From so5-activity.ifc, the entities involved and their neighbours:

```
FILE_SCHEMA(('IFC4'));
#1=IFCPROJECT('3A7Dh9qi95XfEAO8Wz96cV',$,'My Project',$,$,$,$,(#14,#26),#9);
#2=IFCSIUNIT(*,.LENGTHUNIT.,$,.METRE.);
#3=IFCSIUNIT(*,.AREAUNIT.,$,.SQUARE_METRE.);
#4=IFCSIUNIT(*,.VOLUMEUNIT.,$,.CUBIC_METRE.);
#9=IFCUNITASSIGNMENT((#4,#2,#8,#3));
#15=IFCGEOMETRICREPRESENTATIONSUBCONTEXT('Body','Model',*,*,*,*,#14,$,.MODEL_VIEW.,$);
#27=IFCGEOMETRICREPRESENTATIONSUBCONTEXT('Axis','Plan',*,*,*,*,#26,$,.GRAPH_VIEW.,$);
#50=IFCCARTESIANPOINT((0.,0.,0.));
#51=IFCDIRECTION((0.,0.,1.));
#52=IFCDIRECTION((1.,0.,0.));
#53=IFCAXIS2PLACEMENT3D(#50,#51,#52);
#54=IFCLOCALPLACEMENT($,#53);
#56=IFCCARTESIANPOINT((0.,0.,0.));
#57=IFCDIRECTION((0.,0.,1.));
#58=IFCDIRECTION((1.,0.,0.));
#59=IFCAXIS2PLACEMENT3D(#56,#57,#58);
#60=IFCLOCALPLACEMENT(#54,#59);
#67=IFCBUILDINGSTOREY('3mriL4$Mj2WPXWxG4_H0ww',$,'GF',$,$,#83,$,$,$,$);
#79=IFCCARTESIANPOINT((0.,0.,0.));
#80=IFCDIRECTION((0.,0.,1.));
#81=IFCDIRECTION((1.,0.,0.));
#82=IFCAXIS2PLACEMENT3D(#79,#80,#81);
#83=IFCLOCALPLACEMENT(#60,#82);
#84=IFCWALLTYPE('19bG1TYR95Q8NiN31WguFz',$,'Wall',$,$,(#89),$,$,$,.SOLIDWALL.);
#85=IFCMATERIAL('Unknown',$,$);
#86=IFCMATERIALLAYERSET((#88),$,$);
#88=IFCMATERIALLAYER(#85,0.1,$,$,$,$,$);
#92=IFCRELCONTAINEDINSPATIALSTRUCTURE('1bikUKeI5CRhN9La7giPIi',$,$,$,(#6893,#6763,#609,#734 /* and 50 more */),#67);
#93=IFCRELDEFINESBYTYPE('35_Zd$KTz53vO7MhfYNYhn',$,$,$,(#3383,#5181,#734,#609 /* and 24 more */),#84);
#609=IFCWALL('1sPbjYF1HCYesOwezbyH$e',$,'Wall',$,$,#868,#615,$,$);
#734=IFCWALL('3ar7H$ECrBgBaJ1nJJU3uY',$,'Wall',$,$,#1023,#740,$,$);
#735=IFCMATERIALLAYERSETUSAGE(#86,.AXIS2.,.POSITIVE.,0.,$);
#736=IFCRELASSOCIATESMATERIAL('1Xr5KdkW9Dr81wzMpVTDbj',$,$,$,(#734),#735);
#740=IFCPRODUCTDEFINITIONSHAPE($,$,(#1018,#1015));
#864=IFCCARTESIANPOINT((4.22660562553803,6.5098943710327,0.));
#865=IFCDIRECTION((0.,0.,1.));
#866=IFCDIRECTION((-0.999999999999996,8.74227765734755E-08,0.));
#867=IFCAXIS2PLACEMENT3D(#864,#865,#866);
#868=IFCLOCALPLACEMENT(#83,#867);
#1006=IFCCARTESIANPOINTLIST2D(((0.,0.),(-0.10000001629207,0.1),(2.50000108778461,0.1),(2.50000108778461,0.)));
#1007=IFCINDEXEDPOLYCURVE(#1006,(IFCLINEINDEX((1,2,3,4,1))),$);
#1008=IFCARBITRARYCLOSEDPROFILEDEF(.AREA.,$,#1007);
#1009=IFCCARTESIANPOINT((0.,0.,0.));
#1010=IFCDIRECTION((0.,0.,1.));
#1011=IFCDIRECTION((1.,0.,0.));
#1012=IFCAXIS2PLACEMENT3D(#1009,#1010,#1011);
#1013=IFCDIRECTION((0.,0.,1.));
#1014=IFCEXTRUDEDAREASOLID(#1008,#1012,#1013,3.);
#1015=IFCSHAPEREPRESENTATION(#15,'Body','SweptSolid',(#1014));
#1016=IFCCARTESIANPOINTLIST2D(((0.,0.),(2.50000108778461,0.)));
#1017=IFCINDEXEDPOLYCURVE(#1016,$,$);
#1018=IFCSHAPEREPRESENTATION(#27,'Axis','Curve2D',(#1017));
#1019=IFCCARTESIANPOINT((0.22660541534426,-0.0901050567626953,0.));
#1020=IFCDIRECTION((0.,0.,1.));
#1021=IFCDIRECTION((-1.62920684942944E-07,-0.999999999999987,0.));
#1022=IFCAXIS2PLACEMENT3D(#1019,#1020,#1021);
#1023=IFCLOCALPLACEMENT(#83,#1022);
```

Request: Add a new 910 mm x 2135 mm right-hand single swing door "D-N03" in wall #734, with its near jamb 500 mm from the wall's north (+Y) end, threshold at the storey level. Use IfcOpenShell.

```python
import numpy as np
import ifcopenshell
import ifcopenshell.api.feature
import ifcopenshell.api.geometry
import ifcopenshell.api.root
import ifcopenshell.api.spatial
import ifcopenshell.geom
import ifcopenshell.util.element
import ifcopenshell.util.placement
import ifcopenshell.util.representation
import ifcopenshell.util.shape
import ifcopenshell.util.unit

model = ifcopenshell.open("so5-activity.ifc")
unit_scale = ifcopenshell.util.unit.calculate_unit_scale(model)
settings = ifcopenshell.geom.settings()


def volume(element):
    """Net volume in cubic metres, openings subtracted."""
    shape = ifcopenshell.geom.create_shape(settings, element)
    return ifcopenshell.util.shape.get_volume(shape.geometry)


wall = model.by_id(734)
storey = ifcopenshell.util.element.get_container(wall, ifc_class="IfcBuildingStorey")
context = ifcopenshell.util.representation.get_context(model, "Model", "Body", "MODEL_VIEW")
before = volume(wall)

width, height, from_end, sill = 0.91, 2.135, 0.5, 0.0  # metres

# The wall runs along its own X axis, and the end named is its -X end.
wall_shape = ifcopenshell.geom.create_shape(settings, wall)
x, y, z = ifcopenshell.util.shape.get_vertices(wall_shape.geometry).T
start = x.min() + from_end
face, thickness = float(y.min()), float(y.max() - y.min())
wall_matrix = ifcopenshell.util.placement.get_local_placement(wall.ObjectPlacement)
level = ifcopenshell.util.placement.get_local_placement(storey.ObjectPlacement)[2, 3]


def in_wall(x, y):
    """Placement at x, y metres in the wall's axes, at sill height."""
    matrix = wall_matrix.copy()
    matrix[:, 3] = wall_matrix @ np.array([x / unit_scale, y / unit_scale, 0.0, 1.0])
    matrix[2, 3] = level + sill / unit_scale
    return matrix


# Opening: a box that overshoots both wall faces by 50 mm.
opening = ifcopenshell.api.root.create_entity(model, ifc_class="IfcOpeningElement", predefined_type="OPENING")
box = ifcopenshell.api.geometry.add_wall_representation(
    model, context=context, length=width, height=height, thickness=thickness + 0.1
)
ifcopenshell.api.geometry.assign_representation(model, product=opening, representation=box)
ifcopenshell.api.geometry.edit_object_placement(model, product=opening, matrix=in_wall(start, face - 0.05), is_si=False)
ifcopenshell.api.feature.add_feature(model, feature=opening, element=wall)

door = ifcopenshell.api.root.create_entity(model, ifc_class="IfcDoor", name="D-N03", predefined_type="DOOR")
door.OverallWidth, door.OverallHeight = width / unit_scale, height / unit_scale
door.OperationType = "SINGLE_SWING_RIGHT"
body = ifcopenshell.api.geometry.add_door_representation(
    model,
    context=context,
    overall_width=door.OverallWidth,
    overall_height=door.OverallHeight,
    operation_type="SINGLE_SWING_RIGHT",
    lining_properties={"LiningDepth": thickness / unit_scale, "ThresholdDepth": thickness / unit_scale},
)
ifcopenshell.api.geometry.assign_representation(model, product=door, representation=body)
ifcopenshell.api.spatial.assign_container(model, products=[door], relating_structure=storey)
ifcopenshell.api.feature.add_filling(model, opening=opening, element=door)

# The lining spans the wall, so the door starts at the wall face.
ifcopenshell.api.geometry.edit_object_placement(model, product=door, matrix=in_wall(start, face), is_si=False)

after = volume(wall)

print(f"wall volume {before:.3f} -> {after:.3f} m3")

model.write("so5-activity_edited.ifc")
```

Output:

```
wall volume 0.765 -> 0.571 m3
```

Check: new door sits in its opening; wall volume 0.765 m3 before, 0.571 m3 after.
